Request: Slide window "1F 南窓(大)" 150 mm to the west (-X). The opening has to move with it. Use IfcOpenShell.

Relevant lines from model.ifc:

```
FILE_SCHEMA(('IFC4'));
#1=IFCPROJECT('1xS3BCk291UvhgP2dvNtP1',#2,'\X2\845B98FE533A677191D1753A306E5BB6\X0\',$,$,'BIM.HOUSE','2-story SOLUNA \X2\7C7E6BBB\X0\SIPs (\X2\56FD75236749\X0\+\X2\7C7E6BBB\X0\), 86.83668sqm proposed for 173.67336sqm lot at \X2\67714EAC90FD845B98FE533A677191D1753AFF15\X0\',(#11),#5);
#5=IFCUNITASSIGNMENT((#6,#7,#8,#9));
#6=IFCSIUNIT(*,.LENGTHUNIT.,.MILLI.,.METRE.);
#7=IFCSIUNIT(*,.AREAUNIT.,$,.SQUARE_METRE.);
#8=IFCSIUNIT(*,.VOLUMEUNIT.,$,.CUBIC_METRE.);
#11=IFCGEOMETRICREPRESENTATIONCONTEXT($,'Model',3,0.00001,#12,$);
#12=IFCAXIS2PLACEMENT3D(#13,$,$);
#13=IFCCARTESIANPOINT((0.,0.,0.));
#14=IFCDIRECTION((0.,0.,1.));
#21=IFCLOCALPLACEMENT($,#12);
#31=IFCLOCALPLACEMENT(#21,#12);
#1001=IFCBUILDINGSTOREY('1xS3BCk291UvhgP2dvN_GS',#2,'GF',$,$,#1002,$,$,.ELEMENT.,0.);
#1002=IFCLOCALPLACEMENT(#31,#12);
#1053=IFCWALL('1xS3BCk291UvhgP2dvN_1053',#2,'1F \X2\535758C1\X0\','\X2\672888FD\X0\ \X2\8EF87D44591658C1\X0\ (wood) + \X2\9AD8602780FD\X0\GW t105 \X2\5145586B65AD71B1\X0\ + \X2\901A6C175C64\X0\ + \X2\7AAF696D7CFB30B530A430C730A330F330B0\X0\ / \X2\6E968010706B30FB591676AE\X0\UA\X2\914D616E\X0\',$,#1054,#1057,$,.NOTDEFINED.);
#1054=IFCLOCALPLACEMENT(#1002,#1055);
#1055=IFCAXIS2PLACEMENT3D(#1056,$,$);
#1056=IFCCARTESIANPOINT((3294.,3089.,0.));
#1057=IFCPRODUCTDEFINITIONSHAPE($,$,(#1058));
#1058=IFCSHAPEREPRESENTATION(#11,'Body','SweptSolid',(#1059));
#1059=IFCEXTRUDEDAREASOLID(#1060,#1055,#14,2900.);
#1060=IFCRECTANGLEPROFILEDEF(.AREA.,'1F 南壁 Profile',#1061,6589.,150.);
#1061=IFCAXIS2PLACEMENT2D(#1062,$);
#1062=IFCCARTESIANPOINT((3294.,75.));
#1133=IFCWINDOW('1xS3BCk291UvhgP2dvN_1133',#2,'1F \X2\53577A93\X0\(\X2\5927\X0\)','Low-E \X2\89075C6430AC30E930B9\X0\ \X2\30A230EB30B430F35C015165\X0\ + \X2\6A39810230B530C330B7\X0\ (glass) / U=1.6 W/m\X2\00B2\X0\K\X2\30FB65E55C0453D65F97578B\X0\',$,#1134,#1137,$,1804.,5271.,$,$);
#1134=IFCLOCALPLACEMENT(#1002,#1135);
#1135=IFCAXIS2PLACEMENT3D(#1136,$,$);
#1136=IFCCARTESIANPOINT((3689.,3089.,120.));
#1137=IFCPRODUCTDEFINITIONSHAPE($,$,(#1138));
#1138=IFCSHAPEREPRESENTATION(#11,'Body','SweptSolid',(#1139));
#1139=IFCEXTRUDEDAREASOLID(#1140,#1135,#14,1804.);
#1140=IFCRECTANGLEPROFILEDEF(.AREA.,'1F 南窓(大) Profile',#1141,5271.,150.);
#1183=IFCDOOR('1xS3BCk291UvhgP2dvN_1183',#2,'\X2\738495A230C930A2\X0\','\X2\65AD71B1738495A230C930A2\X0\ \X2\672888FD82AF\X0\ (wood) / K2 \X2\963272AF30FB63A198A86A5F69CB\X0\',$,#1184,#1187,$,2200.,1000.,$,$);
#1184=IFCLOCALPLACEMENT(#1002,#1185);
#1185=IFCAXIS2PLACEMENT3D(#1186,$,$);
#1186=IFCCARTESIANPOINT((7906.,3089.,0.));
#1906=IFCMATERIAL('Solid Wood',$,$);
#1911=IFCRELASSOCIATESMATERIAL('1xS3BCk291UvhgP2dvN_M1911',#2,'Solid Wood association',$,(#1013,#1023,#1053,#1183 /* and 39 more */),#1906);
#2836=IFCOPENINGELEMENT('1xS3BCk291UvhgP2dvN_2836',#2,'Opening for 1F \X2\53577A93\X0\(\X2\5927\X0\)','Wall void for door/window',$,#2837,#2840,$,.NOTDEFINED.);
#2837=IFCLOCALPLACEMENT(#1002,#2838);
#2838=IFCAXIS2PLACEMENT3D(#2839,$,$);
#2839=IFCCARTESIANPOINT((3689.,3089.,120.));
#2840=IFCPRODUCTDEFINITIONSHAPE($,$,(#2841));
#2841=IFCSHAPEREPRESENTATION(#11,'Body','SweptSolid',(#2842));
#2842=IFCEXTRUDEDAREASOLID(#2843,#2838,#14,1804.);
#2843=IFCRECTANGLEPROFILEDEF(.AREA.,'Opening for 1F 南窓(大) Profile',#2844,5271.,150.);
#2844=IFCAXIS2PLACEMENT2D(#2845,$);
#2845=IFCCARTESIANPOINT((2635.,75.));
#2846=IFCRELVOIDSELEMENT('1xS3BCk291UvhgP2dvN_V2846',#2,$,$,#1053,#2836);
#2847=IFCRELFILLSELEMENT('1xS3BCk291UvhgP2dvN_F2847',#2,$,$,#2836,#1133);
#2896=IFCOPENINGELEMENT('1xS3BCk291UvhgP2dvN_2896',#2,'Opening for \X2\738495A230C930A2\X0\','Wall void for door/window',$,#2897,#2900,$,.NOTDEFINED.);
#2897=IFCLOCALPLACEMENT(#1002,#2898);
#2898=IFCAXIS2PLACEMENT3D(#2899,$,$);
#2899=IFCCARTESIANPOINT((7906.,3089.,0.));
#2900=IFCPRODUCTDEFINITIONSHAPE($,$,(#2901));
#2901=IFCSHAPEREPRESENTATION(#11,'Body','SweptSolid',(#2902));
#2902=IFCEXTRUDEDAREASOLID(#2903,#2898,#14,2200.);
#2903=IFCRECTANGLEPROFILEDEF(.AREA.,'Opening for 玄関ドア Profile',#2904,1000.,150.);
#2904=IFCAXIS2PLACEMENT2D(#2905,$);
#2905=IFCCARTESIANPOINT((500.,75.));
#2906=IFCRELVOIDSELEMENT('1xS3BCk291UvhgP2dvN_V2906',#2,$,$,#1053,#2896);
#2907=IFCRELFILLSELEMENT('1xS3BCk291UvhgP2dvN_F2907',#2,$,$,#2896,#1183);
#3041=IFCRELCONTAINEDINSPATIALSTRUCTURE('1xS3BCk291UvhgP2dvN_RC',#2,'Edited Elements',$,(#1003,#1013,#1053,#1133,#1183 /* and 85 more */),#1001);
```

```python
import ifcopenshell
import ifcopenshell.api.geometry
import ifcopenshell.util.placement

model = ifcopenshell.open("model.ifc")

window = model.by_guid("1xS3BCk291UvhgP2dvN_1133")
opening = window.FillsVoids[0].RelatingOpeningElement
wall = opening.VoidsElements[0].RelatingBuildingElement

wall_matrix = ifcopenshell.util.placement.get_local_placement(wall.ObjectPlacement)
shift = wall_matrix[:3, 0] * -150.0
before = ifcopenshell.util.placement.get_local_placement(window.ObjectPlacement)[:3, 3].copy()

# The window is not placed relative to its opening, so move both.
for product in (opening, window):
    matrix = ifcopenshell.util.placement.get_local_placement(product.ObjectPlacement)
    matrix[:3, 3] += shift
    ifcopenshell.api.geometry.edit_object_placement(model, product=product, matrix=matrix, is_si=False)

after = ifcopenshell.util.placement.get_local_placement(window.ObjectPlacement)[:3, 3]
print("window moved by", (after - before).round(3) + 0.0)

model.write("model_rev.ifc")
```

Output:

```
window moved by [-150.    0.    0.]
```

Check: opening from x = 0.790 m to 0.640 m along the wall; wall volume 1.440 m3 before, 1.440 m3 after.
